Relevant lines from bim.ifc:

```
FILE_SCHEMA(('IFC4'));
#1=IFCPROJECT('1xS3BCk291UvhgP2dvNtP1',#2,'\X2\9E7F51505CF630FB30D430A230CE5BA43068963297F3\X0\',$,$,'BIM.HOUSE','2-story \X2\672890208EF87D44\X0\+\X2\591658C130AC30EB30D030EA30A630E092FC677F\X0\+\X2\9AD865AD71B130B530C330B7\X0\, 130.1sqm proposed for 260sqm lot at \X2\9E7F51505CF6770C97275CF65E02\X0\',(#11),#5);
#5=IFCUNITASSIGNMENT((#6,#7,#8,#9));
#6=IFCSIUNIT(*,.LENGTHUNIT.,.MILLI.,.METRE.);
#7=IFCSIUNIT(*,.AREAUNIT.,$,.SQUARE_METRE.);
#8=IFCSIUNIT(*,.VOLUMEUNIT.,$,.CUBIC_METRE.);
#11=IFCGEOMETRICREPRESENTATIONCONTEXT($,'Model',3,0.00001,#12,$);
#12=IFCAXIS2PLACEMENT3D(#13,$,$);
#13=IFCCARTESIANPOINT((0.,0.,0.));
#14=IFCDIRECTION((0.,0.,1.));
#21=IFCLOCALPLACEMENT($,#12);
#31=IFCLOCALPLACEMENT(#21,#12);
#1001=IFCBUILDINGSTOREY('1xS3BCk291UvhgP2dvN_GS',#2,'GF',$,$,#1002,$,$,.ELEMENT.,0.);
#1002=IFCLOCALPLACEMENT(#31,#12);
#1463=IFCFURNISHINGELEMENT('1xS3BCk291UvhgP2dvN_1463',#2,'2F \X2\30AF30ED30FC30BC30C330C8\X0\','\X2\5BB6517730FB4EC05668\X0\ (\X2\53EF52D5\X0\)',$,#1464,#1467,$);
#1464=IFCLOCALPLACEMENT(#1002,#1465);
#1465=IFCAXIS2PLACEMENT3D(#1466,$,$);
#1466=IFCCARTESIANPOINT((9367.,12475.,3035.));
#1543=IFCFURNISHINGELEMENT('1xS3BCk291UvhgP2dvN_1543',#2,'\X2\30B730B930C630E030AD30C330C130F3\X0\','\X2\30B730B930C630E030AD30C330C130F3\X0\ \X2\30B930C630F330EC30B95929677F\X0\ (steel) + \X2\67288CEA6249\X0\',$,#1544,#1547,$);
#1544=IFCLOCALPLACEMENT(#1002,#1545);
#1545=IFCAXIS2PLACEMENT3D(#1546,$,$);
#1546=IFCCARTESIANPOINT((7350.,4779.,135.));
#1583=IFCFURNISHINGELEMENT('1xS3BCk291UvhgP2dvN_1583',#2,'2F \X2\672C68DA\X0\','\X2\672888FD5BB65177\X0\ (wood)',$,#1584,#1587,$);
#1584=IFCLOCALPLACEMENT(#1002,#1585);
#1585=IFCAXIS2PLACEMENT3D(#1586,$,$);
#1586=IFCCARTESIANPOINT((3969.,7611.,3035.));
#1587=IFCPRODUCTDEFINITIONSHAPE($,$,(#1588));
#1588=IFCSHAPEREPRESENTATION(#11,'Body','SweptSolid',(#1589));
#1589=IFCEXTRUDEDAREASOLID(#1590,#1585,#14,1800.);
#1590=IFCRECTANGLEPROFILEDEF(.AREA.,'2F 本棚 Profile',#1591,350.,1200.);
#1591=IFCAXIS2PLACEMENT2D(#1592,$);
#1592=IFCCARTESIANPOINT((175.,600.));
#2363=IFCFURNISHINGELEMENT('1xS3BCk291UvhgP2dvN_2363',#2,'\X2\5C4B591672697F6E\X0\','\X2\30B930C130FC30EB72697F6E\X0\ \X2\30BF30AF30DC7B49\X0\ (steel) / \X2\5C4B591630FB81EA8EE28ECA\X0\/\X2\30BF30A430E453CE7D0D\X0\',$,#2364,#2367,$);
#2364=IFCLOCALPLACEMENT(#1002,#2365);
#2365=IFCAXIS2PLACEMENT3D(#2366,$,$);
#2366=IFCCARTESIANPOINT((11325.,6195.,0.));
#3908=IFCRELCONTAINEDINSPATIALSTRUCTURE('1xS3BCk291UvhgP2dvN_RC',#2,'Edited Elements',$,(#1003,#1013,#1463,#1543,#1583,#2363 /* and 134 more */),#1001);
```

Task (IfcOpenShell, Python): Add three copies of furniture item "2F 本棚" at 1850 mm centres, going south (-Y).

```python
import numpy as np
import ifcopenshell
import ifcopenshell.api.geometry
import ifcopenshell.api.root
import ifcopenshell.util.element
import ifcopenshell.util.placement
import ifcopenshell.util.unit

model = ifcopenshell.open("bim.ifc")
unit_scale = ifcopenshell.util.unit.calculate_unit_scale(model)


def reuse_history(source, copy):
    """copy_class also copies each property set's owner history, people and application; keep the originals."""
    for rel in copy.IsDefinedBy:
        if rel.is_a("IfcRelDefinesByProperties") and (history := rel.RelatingPropertyDefinition.OwnerHistory):
            rel.RelatingPropertyDefinition.OwnerHistory = source.OwnerHistory
            ifcopenshell.util.element.remove_deep2(model, history)


source = model.by_id(1583)
base = ifcopenshell.util.placement.get_local_placement(source.ObjectPlacement)
step = np.array([0.0, -1.0, 0.0]) * 1.85 / unit_scale

for i in range(1, 4):
    copy = ifcopenshell.api.root.copy_class(model, product=source)
    copy.Representation = ifcopenshell.util.element.copy_deep(
        model, source.Representation, exclude=["IfcGeometricRepresentationContext", "IfcRepresentationMap"]
    )
    reuse_history(source, copy)
    matrix = base.copy()
    matrix[:3, 3] += i * step
    print("added at", matrix[:3, 3].round(3) + 0.0)
    ifcopenshell.api.geometry.edit_object_placement(model, product=copy, matrix=matrix, is_si=False)

model.write("bim_v2.ifc")
```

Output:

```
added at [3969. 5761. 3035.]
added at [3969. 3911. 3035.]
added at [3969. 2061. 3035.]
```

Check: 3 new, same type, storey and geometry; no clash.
